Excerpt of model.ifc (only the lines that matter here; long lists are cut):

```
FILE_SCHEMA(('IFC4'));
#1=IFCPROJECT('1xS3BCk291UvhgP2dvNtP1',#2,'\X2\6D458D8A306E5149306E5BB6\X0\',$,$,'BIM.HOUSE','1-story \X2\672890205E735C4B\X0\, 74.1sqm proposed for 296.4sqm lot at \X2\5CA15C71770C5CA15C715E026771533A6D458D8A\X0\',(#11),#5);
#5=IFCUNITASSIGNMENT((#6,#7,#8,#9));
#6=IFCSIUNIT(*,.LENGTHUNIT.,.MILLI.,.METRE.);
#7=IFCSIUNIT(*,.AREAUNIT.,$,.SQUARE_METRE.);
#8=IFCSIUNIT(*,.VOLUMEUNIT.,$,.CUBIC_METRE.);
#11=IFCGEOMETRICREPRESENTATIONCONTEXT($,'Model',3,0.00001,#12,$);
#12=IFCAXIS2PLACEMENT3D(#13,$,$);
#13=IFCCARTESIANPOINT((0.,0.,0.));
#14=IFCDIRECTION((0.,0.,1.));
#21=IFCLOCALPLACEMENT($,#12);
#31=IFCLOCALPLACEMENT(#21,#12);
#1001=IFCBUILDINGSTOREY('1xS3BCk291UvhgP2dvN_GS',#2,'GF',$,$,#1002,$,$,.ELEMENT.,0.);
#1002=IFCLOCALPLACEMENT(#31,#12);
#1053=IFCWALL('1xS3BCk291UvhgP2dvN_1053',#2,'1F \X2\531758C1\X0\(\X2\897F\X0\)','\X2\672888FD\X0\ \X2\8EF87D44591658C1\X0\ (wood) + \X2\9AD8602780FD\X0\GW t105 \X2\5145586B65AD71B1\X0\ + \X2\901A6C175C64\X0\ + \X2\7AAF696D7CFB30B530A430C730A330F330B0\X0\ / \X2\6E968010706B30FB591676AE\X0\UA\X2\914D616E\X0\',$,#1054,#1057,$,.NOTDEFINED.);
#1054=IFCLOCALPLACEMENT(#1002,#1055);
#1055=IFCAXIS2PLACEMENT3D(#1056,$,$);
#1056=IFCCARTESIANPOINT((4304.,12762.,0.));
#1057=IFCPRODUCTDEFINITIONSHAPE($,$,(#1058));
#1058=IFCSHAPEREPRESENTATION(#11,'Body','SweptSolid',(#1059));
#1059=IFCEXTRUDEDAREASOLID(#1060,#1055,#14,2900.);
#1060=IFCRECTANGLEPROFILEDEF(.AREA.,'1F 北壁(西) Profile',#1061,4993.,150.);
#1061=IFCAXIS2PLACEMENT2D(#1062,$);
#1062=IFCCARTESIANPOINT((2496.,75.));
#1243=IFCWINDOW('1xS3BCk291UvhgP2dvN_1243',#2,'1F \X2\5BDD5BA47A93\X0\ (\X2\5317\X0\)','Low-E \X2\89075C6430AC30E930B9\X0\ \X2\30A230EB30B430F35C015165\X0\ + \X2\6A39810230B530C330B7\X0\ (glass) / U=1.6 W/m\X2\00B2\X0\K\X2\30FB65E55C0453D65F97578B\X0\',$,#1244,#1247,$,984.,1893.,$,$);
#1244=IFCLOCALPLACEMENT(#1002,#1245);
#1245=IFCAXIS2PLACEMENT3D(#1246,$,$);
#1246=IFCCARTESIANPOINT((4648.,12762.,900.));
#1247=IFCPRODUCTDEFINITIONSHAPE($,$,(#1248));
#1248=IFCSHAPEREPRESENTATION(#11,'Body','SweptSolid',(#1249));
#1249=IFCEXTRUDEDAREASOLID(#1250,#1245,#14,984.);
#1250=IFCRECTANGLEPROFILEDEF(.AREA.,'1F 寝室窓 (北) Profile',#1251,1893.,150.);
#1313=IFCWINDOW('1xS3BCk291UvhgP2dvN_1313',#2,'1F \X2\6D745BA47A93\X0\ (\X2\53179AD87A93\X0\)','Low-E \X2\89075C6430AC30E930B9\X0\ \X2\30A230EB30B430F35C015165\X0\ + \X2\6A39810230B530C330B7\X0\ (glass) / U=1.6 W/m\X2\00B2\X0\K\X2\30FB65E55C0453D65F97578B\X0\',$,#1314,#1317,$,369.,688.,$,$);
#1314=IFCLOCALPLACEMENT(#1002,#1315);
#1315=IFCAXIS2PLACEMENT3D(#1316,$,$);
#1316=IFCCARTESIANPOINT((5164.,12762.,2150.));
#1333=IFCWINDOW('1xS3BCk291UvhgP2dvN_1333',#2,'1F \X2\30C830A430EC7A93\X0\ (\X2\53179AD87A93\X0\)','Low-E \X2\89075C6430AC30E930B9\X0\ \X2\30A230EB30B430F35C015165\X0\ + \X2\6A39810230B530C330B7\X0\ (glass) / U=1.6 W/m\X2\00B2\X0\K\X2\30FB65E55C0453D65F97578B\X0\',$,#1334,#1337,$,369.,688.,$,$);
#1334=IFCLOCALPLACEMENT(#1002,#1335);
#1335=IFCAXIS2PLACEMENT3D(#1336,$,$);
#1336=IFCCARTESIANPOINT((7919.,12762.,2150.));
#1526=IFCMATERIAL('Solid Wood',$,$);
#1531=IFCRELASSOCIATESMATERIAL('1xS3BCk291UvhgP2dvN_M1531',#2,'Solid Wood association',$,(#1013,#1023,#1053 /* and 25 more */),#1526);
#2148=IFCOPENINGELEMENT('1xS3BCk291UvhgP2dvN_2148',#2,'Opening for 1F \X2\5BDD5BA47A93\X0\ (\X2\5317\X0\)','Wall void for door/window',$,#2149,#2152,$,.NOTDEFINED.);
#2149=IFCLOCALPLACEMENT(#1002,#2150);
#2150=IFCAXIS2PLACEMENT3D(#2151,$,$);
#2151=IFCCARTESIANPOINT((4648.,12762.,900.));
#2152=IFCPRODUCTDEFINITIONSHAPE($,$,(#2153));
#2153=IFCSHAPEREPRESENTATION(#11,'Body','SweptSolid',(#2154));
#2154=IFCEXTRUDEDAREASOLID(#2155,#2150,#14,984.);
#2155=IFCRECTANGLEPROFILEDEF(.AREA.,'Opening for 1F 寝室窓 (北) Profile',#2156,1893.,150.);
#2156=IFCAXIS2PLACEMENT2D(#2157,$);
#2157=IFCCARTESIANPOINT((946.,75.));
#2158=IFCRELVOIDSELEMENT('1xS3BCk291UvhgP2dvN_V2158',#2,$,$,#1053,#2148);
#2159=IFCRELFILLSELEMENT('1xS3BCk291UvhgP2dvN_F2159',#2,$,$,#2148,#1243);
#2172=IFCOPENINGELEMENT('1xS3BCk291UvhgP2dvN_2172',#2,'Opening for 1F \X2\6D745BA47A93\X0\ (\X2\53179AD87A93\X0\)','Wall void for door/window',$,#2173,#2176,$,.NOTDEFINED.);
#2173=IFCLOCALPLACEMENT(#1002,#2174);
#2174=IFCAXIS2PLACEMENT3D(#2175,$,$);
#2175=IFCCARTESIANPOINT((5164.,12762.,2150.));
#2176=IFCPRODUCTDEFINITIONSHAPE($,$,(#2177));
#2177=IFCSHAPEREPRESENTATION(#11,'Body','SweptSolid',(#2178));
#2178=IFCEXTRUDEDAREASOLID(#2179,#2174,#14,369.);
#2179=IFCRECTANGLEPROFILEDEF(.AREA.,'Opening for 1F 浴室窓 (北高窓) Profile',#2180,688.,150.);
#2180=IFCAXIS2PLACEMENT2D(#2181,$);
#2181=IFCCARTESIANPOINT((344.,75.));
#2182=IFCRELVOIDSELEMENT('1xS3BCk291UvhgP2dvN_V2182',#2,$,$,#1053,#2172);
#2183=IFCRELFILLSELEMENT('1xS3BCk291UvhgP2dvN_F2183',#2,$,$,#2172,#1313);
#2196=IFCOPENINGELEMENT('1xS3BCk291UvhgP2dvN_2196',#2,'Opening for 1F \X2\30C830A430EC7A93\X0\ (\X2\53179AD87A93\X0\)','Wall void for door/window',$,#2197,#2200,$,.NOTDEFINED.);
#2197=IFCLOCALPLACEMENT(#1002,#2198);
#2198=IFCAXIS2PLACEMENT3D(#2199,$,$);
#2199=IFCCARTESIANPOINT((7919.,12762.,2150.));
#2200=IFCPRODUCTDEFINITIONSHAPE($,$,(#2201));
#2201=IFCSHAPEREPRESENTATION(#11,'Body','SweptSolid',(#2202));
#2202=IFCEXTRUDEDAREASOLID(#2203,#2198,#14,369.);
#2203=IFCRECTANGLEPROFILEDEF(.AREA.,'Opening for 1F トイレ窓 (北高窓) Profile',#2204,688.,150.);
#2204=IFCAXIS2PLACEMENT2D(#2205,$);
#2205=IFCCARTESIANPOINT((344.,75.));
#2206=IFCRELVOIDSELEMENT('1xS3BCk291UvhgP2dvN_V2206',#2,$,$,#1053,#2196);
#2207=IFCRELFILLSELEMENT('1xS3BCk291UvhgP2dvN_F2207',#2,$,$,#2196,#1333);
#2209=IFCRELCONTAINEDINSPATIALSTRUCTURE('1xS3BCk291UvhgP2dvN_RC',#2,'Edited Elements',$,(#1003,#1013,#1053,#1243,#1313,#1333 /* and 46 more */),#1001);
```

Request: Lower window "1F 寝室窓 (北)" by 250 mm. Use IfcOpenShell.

```python
import numpy as np
import ifcopenshell
import ifcopenshell.api.geometry
import ifcopenshell.util.placement
import ifcopenshell.util.unit

model = ifcopenshell.open("model.ifc")
unit_scale = ifcopenshell.util.unit.calculate_unit_scale(model)

window = model.by_id(1243)
opening = window.FillsVoids[0].RelatingOpeningElement
dz = -0.25 / unit_scale

shift = np.array([0.0, 0.0, dz])
# The window is not placed relative to its opening, so move both.
for product in (opening, window):
    matrix = ifcopenshell.util.placement.get_local_placement(product.ObjectPlacement)
    matrix[:3, 3] += shift
    ifcopenshell.api.geometry.edit_object_placement(model, product=product, matrix=matrix, is_si=False)

print(f"moved by {dz * unit_scale:+.3f} m")

model.write("model_v2.ifc")
```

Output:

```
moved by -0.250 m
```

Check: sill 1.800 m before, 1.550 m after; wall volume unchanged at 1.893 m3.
